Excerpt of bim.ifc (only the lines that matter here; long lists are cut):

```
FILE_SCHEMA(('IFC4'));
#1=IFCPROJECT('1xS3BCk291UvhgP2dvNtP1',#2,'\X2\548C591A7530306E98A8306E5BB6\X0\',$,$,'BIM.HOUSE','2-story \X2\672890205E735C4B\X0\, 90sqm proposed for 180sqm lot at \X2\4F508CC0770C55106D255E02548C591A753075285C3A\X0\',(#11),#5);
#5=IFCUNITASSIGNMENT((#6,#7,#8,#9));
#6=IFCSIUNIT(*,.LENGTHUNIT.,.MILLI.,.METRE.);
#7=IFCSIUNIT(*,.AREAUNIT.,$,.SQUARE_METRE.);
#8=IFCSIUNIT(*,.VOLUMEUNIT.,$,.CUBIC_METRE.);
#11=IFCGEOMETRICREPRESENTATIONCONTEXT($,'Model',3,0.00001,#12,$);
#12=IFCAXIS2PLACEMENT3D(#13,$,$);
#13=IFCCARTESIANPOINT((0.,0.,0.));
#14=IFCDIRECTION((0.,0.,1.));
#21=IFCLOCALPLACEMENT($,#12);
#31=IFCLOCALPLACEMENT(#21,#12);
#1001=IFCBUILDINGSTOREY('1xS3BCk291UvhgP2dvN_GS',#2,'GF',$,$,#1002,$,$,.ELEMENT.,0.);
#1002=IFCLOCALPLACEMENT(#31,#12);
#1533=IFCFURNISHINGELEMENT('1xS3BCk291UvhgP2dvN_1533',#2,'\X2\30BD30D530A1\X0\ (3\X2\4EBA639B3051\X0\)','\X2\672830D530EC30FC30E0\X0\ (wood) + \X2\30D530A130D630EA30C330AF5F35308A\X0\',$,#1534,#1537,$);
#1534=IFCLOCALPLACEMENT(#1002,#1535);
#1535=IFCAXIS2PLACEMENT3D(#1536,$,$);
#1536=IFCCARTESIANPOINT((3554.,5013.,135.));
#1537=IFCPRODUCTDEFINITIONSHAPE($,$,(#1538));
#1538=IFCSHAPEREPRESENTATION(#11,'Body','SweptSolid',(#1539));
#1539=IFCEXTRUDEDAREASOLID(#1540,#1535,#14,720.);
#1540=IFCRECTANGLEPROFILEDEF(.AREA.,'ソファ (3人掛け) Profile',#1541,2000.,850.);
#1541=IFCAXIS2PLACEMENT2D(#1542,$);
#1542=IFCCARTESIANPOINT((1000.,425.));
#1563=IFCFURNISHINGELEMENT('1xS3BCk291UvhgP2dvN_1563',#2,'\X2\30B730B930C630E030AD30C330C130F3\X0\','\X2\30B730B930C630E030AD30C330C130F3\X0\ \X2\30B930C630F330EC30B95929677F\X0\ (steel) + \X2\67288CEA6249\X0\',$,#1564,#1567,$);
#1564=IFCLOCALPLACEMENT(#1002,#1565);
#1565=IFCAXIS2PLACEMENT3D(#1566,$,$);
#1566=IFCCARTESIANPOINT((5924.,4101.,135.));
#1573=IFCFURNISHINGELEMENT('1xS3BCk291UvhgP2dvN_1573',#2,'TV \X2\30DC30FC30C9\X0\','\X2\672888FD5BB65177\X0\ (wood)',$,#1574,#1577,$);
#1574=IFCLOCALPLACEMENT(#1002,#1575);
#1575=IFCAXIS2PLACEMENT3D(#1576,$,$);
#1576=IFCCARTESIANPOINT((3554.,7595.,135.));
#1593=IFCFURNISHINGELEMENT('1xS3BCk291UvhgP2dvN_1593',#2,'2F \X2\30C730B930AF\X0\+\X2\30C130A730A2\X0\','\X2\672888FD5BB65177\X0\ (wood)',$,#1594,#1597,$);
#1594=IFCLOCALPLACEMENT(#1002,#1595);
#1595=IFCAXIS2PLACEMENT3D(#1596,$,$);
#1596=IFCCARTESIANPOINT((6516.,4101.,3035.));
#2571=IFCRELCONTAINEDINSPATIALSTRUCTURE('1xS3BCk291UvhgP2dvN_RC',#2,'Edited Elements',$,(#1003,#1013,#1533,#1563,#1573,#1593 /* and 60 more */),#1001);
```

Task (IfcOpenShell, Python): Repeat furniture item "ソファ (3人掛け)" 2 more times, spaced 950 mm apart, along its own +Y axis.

```python
import ifcopenshell
import ifcopenshell.api.geometry
import ifcopenshell.api.root
import ifcopenshell.util.element
import ifcopenshell.util.placement

model = ifcopenshell.open("bim.ifc")


def reuse_history(source, copy):
    """copy_class also copies each property set's owner history, people and application; keep the originals."""
    for rel in copy.IsDefinedBy:
        if rel.is_a("IfcRelDefinesByProperties") and (history := rel.RelatingPropertyDefinition.OwnerHistory):
            rel.RelatingPropertyDefinition.OwnerHistory = source.OwnerHistory
            ifcopenshell.util.element.remove_deep2(model, history)


source = model.by_id(1533)
base = ifcopenshell.util.placement.get_local_placement(source.ObjectPlacement)
step = base[:3, 1] * 950.0

for i in range(1, 3):
    copy = ifcopenshell.api.root.copy_class(model, product=source)
    copy.Representation = ifcopenshell.util.element.copy_deep(
        model, source.Representation, exclude=["IfcGeometricRepresentationContext", "IfcRepresentationMap"]
    )
    reuse_history(source, copy)
    matrix = base.copy()
    matrix[:3, 3] += i * step
    print("added at", matrix[:3, 3].round(3) + 0.0)
    ifcopenshell.api.geometry.edit_object_placement(model, product=copy, matrix=matrix, is_si=False)

model.write("bim-out.ifc")
```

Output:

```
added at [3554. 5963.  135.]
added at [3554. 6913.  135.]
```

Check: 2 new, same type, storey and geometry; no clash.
